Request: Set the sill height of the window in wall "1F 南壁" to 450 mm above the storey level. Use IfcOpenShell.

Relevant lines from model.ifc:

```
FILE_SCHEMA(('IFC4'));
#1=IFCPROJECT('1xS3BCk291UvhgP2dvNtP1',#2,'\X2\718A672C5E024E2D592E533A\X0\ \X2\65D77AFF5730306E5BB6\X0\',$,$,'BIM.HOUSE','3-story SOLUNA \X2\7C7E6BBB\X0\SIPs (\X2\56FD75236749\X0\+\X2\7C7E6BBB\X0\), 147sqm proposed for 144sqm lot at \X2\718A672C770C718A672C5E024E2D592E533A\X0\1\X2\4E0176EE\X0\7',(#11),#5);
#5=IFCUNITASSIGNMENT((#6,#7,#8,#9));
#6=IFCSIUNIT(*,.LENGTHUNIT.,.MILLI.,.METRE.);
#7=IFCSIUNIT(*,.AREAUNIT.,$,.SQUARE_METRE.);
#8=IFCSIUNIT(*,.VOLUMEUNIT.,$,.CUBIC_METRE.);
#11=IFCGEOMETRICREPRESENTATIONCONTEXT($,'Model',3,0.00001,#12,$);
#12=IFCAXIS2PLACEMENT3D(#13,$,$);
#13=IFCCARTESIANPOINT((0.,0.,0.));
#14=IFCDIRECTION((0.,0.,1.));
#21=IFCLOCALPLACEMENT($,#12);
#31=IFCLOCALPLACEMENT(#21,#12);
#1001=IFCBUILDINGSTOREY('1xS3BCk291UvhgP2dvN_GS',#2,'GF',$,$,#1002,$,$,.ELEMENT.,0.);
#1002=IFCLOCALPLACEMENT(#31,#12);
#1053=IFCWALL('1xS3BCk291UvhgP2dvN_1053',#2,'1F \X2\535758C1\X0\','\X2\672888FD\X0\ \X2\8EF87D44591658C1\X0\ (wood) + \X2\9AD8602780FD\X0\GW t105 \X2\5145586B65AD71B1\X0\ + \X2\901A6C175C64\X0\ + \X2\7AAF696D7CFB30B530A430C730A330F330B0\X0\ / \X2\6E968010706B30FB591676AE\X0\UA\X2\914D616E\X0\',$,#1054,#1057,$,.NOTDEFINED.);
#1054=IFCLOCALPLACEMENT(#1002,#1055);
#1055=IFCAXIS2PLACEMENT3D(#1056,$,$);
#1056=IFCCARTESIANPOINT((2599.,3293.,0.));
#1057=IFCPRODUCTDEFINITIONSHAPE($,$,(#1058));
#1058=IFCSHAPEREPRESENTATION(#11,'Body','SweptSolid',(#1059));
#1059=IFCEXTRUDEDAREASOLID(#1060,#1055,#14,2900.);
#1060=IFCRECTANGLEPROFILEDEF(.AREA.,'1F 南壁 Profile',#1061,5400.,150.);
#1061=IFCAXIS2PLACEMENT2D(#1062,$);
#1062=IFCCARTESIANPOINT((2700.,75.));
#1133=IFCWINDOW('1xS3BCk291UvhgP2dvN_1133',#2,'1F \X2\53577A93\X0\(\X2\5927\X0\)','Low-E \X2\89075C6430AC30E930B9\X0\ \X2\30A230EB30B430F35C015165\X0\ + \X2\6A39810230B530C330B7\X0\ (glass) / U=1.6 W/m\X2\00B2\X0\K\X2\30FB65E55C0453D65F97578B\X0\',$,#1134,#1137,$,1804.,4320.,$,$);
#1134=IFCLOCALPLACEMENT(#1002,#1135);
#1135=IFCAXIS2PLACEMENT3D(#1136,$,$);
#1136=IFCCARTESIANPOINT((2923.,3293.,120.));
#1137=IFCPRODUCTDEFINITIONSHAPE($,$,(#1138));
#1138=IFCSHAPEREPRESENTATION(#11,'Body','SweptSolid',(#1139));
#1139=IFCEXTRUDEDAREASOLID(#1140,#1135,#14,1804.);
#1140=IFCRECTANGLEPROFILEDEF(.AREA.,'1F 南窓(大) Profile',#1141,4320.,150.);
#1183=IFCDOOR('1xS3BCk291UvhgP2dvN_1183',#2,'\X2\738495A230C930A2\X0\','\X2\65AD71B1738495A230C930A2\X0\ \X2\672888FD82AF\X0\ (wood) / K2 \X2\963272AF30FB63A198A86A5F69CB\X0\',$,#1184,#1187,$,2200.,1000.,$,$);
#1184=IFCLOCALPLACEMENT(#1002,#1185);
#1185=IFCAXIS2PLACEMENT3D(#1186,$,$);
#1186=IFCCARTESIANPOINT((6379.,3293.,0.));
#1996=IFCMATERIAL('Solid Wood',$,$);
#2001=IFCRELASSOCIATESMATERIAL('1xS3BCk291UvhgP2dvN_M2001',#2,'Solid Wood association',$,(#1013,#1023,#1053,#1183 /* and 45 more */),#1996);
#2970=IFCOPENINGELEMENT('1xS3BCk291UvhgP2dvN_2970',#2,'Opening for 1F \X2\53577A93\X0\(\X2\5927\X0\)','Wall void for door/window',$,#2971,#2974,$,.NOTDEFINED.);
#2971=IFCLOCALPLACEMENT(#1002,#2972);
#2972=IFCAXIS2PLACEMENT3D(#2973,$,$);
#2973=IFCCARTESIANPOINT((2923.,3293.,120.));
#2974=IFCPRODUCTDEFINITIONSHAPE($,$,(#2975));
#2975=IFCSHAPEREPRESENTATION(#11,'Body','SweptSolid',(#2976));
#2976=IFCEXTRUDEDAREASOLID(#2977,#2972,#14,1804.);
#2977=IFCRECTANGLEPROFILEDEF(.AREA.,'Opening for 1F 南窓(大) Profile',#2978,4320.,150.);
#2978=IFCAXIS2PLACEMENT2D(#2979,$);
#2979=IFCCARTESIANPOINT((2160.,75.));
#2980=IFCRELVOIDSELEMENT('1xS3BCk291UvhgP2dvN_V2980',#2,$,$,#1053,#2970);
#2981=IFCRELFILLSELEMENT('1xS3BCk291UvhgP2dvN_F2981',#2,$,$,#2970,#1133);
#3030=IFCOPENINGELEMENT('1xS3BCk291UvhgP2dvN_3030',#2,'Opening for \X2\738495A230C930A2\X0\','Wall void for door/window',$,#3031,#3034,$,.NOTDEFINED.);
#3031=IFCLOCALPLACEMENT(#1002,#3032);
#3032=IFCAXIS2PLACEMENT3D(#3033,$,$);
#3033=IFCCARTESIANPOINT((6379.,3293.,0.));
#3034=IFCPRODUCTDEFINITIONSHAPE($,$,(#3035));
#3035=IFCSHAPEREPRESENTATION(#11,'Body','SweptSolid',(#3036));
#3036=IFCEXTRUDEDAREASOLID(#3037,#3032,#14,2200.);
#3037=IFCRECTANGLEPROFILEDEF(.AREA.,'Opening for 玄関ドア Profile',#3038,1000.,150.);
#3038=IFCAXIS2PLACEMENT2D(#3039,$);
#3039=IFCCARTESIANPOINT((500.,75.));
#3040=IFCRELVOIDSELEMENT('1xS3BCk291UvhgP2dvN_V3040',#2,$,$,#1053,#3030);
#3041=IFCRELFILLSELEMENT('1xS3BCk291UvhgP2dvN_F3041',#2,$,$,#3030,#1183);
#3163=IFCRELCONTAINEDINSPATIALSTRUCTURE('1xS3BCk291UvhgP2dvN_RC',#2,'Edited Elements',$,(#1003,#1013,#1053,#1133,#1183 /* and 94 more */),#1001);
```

```python
import numpy as np
import ifcopenshell
import ifcopenshell.api.geometry
import ifcopenshell.geom
import ifcopenshell.util.element
import ifcopenshell.util.placement
import ifcopenshell.util.shape
import ifcopenshell.util.unit

model = ifcopenshell.open("model.ifc")
unit_scale = ifcopenshell.util.unit.calculate_unit_scale(model)

window = model.by_guid("1xS3BCk291UvhgP2dvN_1133")
opening = window.FillsVoids[0].RelatingOpeningElement
storey = ifcopenshell.util.element.get_container(window, ifc_class="IfcBuildingStorey")
level = ifcopenshell.util.placement.get_local_placement(storey.ObjectPlacement)[2, 3]

# The opening's origin need not be at the sill, so measure its lowest point.
shape = ifcopenshell.geom.create_shape(ifcopenshell.geom.settings(), opening)
bottom = ifcopenshell.util.shape.get_shape_bottom_elevation(shape, shape.geometry) / unit_scale
dz = level + 0.45 / unit_scale - bottom

shift = np.array([0.0, 0.0, dz])
# The window is not placed relative to its opening, so move both.
for product in (opening, window):
    matrix = ifcopenshell.util.placement.get_local_placement(product.ObjectPlacement)
    matrix[:3, 3] += shift
    ifcopenshell.api.geometry.edit_object_placement(model, product=product, matrix=matrix, is_si=False)

print(f"moved by {dz * unit_scale:+.3f} m")

model.write("model_rev.ifc")
```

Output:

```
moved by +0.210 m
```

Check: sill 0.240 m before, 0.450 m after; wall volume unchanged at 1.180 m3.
